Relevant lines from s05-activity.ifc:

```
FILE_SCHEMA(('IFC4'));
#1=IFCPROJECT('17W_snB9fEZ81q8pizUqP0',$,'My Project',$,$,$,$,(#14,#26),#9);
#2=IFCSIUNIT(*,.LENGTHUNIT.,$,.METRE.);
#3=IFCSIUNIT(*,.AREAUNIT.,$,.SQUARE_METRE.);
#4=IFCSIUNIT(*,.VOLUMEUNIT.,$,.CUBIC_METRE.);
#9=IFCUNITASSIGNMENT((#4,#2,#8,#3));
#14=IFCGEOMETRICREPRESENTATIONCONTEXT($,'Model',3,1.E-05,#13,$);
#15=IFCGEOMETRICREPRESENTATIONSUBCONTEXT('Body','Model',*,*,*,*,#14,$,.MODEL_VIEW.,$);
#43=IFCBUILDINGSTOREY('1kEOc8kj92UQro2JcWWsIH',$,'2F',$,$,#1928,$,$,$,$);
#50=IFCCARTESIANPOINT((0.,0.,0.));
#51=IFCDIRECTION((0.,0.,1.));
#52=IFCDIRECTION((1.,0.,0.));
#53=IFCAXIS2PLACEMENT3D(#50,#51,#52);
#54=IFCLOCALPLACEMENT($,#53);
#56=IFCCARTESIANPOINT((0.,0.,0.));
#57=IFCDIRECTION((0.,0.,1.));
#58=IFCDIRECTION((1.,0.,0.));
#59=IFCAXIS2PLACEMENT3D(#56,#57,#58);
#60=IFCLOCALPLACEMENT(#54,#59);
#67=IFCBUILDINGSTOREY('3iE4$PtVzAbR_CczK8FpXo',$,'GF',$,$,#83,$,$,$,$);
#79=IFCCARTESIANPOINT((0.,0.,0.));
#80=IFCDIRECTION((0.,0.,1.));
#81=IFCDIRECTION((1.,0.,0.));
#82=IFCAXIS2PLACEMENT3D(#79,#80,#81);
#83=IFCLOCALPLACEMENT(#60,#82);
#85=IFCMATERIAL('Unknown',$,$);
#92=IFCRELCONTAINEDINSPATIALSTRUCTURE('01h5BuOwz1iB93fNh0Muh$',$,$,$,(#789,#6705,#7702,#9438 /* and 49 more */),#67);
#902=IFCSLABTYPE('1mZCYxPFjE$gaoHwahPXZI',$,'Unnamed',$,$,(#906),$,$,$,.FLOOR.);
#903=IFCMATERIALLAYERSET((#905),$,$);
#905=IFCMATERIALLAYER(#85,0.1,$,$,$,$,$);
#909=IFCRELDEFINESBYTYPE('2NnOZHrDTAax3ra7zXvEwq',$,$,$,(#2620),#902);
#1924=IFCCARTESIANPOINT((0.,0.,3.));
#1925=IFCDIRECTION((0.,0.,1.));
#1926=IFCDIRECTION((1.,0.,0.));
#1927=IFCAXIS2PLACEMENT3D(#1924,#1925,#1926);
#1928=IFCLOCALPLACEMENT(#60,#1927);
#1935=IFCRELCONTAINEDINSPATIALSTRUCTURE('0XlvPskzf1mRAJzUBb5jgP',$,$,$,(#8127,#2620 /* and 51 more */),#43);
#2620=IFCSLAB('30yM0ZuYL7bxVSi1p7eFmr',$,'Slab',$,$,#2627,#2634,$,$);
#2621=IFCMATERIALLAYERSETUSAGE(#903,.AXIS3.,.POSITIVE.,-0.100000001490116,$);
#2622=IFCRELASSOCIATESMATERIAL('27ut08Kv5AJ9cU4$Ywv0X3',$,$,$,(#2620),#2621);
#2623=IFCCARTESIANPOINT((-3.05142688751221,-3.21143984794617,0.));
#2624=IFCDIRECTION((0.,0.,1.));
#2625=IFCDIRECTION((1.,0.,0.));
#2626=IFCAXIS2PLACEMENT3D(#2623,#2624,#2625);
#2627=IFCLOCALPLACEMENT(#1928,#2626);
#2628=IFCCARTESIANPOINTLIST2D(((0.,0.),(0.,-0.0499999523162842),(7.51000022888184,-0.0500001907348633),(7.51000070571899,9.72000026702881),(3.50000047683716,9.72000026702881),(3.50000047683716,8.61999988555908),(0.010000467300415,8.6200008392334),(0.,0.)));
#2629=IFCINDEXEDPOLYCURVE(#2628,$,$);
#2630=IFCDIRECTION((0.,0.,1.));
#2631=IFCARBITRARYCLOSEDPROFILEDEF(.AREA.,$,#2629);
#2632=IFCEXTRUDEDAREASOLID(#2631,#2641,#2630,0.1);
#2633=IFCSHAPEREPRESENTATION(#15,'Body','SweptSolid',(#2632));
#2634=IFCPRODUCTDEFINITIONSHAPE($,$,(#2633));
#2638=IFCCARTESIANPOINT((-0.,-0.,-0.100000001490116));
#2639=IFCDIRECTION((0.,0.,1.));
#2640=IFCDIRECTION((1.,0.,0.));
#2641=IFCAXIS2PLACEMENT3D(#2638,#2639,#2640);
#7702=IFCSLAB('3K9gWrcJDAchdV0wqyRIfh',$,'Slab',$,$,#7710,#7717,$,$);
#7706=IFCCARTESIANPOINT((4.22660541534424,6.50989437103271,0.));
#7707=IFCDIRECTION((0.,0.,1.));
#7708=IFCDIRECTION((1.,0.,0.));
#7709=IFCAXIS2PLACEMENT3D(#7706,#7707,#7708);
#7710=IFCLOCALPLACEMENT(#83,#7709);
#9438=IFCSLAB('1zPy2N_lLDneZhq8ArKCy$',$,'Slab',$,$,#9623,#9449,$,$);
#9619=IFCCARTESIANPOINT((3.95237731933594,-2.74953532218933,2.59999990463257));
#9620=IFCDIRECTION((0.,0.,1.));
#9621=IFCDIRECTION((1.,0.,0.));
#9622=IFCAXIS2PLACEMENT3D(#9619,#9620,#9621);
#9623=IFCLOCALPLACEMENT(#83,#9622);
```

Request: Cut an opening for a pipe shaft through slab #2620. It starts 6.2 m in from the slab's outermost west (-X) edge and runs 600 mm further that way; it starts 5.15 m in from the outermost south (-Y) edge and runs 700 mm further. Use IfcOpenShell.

```python
import numpy as np
import ifcopenshell
import ifcopenshell.api.feature
import ifcopenshell.api.geometry
import ifcopenshell.api.root
import ifcopenshell.geom
import ifcopenshell.util.placement
import ifcopenshell.util.representation
import ifcopenshell.util.shape
import ifcopenshell.util.unit

model = ifcopenshell.open("s05-activity.ifc")
unit_scale = ifcopenshell.util.unit.calculate_unit_scale(model)
settings = ifcopenshell.geom.settings()


def volume(element):
    """Net volume in cubic metres, openings subtracted."""
    shape = ifcopenshell.geom.create_shape(settings, element)
    return ifcopenshell.util.shape.get_volume(shape.geometry)


slab = model.by_guid("30yM0ZuYL7bxVSi1p7eFmr")
before = volume(slab)

# Extent in the slab's own axes, in metres. The edges named are its -X and -Y sides.
slab_shape = ifcopenshell.geom.create_shape(settings, slab)
vertices = ifcopenshell.util.shape.get_vertices(slab_shape.geometry)
x_min, y_min, bottom = vertices.min(axis=0)
top = vertices[:, 2].max()

opening = ifcopenshell.api.root.create_entity(model, ifc_class="IfcOpeningElement", name="Pipe shaft opening", predefined_type="OPENING")
context = ifcopenshell.util.representation.get_context(model, "Model", "Body", "MODEL_VIEW")
width, depth = 0.6, 0.7
outline = [(0.0, 0.0), (width, 0.0), (width, depth), (0.0, depth), (0.0, 0.0)]
# Overshoot both faces by 50 mm so the cut is clean.
shape = ifcopenshell.api.geometry.add_slab_representation(
    model, context=context, depth=top - bottom + 0.1, polyline=outline
)
ifcopenshell.api.geometry.assign_representation(model, product=opening, representation=shape)

matrix = ifcopenshell.util.placement.get_local_placement(slab.ObjectPlacement)
matrix[:, 3] = matrix @ np.append(np.array([x_min + 6.2, y_min + 5.15, bottom - 0.05]) / unit_scale, 1.0)
ifcopenshell.api.geometry.edit_object_placement(model, product=opening, matrix=matrix, is_si=False)
ifcopenshell.api.feature.add_feature(model, feature=opening, element=slab)

after = volume(slab)

print(f"slab volume {before:.3f} -> {after:.3f} m3")

model.write("s05-activity_v2.ifc")
```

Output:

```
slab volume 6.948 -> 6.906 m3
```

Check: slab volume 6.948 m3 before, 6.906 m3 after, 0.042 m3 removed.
